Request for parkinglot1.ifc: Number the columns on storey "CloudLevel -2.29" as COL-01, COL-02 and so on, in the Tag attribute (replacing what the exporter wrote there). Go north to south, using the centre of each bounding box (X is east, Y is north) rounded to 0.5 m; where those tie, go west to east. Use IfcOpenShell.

First a look at what the model holds.

```python
import ifcopenshell
import ifcopenshell.util.element
import ifcopenshell.util.placement

model = ifcopenshell.open("parkinglot1.ifc")
print(model.schema)
storey = next(s for s in model.by_type("IfcBuildingStorey") if s.Name == "CloudLevel -2.29")
columns = [e for e in ifcopenshell.util.element.get_decomposition(storey) if e.is_a("IfcColumn")]
for e in sorted(columns, key=lambda e: e.id()):
    origin = ifcopenshell.util.placement.get_local_placement(e.ObjectPlacement)[:3, 3]
    print(e.id(), e.Tag, e.Name, origin.round(2) + 0.0, sep=" | ")
```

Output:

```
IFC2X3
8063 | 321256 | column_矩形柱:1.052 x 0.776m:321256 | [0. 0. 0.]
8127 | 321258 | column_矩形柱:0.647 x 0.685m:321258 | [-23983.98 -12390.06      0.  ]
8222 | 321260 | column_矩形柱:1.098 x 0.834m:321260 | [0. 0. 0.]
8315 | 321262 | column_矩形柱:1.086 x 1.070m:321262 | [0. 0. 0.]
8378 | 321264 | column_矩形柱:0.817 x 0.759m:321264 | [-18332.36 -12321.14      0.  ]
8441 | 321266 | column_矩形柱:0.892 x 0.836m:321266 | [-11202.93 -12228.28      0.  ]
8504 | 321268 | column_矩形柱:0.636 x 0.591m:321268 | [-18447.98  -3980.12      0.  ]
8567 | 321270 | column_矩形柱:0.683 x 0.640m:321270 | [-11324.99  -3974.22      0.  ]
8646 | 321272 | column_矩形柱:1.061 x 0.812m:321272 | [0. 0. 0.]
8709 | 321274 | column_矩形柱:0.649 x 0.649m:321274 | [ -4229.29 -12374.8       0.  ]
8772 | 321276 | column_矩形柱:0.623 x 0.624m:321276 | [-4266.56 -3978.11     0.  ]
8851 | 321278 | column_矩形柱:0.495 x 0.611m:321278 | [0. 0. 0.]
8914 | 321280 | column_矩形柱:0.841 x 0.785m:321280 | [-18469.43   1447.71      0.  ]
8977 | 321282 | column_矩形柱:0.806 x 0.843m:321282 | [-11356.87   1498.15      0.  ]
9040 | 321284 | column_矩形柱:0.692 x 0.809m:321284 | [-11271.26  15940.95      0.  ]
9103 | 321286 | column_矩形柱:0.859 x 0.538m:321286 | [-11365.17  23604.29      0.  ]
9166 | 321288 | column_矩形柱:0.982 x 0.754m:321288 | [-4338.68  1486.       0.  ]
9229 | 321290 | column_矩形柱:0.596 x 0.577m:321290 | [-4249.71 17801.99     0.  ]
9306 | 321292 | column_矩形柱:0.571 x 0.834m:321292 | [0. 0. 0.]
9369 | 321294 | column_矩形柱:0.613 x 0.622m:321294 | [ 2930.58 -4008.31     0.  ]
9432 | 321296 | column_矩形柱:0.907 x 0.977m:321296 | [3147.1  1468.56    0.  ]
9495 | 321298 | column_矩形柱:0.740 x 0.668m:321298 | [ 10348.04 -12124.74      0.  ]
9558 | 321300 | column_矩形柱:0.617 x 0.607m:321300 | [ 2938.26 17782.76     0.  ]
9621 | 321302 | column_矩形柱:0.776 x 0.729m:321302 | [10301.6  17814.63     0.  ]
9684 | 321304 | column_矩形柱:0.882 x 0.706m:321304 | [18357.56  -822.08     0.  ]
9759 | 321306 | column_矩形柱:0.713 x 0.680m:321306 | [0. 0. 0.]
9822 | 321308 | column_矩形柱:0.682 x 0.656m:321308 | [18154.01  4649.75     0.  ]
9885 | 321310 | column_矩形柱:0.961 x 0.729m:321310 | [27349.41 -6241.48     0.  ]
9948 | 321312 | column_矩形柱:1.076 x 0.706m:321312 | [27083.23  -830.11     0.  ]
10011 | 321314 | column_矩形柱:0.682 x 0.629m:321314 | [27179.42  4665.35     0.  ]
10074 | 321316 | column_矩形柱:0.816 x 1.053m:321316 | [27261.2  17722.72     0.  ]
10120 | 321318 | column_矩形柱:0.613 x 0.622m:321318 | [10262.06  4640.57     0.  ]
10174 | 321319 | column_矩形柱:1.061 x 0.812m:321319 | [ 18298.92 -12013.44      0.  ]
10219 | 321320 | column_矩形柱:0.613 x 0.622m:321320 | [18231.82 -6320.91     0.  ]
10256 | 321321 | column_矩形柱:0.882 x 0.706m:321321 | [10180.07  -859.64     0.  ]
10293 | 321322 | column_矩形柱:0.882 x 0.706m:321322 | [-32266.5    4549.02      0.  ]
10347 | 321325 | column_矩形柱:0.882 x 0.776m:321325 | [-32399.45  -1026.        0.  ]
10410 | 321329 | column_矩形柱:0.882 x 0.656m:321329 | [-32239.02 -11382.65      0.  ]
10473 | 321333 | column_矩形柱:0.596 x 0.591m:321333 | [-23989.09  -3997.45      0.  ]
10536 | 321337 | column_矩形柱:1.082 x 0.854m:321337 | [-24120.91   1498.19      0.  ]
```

```python
import ifcopenshell
import ifcopenshell.geom
import ifcopenshell.util.element
import ifcopenshell.util.shape

model = ifcopenshell.open("parkinglot1.ifc")
settings = ifcopenshell.geom.settings()
settings.set("use-world-coords", True)


def centre(element):
    shape = ifcopenshell.geom.create_shape(settings, element)
    return ifcopenshell.util.shape.get_bbox_centroid(shape.geometry)


storey = next(s for s in model.by_type("IfcBuildingStorey") if s.Name == "CloudLevel -2.29")
columns = [e for e in ifcopenshell.util.element.get_decomposition(storey) if e.is_a("IfcColumn")]

# Insertion points can sit at a corner or the storey origin, so sort by the geometry (in metres).
centres = {e: centre(e) for e in columns}
columns.sort(key=lambda e: (-round(centres[e][1] / 0.5), centres[e][0]))

for i, e in enumerate(columns, start=1):
    number = f"COL-{i:02d}"
    e.Tag = number
    print(e.id(), number)

model.write("parkinglot1_rev.ifc")
```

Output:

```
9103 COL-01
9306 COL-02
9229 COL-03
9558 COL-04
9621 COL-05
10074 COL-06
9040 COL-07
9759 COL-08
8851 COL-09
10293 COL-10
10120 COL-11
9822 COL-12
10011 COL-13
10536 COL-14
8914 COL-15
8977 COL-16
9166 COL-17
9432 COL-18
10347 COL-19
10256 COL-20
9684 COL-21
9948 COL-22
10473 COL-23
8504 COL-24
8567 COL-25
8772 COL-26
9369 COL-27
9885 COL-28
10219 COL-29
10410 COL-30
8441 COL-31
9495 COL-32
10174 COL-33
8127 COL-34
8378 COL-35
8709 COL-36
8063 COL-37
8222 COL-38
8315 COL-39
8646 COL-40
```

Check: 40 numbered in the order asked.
